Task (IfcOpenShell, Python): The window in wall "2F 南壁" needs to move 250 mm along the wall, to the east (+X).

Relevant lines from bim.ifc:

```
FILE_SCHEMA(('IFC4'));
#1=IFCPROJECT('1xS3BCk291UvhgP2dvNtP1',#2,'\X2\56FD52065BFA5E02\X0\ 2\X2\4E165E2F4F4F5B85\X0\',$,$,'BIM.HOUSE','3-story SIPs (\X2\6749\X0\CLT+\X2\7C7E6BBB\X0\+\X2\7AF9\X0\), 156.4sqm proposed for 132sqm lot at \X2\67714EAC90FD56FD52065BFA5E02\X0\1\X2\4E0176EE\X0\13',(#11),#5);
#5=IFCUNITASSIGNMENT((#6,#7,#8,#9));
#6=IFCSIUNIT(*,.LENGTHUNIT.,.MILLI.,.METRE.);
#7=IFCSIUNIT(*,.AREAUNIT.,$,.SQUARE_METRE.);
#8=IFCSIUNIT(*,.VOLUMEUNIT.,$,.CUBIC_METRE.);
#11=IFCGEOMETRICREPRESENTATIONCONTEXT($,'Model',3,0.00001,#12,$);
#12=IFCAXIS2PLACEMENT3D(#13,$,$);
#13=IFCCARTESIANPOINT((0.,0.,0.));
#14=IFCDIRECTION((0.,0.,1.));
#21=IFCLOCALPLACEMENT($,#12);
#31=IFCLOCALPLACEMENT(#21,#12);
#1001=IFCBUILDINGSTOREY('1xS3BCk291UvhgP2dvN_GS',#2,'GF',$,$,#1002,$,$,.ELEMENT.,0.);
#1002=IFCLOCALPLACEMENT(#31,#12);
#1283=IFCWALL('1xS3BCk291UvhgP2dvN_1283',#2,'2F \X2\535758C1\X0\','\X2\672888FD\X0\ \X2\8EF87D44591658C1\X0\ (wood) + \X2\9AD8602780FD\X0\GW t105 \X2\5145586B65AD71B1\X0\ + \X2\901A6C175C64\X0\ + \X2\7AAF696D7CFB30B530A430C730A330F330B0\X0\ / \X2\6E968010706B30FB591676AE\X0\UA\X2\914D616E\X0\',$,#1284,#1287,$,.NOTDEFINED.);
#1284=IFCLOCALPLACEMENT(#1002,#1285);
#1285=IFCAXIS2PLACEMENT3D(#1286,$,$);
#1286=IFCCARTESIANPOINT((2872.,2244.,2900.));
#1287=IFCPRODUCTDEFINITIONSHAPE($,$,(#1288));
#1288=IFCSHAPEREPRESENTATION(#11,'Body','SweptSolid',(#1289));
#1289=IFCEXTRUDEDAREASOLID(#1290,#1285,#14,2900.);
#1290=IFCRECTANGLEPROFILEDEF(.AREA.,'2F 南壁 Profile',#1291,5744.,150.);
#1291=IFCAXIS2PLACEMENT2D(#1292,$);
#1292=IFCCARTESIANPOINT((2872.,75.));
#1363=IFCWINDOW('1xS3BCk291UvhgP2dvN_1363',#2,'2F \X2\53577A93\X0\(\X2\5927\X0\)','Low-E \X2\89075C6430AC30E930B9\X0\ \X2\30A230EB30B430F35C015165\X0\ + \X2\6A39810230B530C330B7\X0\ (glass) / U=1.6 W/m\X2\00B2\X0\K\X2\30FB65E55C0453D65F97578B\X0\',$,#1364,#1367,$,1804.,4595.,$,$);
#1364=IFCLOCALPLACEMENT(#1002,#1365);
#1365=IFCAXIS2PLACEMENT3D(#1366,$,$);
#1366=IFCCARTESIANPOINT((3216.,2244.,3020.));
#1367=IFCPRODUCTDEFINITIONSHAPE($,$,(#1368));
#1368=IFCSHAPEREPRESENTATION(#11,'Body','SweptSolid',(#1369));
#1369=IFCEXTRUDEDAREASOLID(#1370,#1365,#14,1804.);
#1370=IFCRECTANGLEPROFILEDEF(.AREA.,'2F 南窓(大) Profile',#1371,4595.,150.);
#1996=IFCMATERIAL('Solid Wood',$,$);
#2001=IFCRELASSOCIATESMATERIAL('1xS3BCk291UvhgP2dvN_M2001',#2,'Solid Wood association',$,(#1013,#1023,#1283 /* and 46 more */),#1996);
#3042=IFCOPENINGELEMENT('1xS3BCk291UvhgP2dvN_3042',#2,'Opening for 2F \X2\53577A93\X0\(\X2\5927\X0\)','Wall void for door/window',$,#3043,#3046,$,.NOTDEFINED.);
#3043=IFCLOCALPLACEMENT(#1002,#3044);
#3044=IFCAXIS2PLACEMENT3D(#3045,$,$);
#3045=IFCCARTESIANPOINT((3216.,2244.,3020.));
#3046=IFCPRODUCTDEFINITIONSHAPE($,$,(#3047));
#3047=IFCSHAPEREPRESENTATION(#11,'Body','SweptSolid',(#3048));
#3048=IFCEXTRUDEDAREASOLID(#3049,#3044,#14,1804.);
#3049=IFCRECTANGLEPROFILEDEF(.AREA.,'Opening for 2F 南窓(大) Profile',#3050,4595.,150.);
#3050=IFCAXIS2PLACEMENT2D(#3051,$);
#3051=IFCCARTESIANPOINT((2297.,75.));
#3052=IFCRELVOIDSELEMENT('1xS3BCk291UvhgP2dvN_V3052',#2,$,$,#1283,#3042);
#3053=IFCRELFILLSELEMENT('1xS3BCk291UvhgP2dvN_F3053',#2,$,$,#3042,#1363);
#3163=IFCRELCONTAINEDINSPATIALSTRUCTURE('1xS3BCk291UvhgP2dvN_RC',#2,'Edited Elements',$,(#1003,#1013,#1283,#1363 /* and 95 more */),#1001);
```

```python
import ifcopenshell
import ifcopenshell.api.geometry
import ifcopenshell.util.placement
import ifcopenshell.util.unit

model = ifcopenshell.open("bim.ifc")
unit_scale = ifcopenshell.util.unit.calculate_unit_scale(model)

window = model.by_guid("1xS3BCk291UvhgP2dvN_1363")
opening = window.FillsVoids[0].RelatingOpeningElement
wall = opening.VoidsElements[0].RelatingBuildingElement

wall_matrix = ifcopenshell.util.placement.get_local_placement(wall.ObjectPlacement)
shift = wall_matrix[:3, 0] * 0.25 / unit_scale
before = ifcopenshell.util.placement.get_local_placement(window.ObjectPlacement)[:3, 3].copy()

# The window is not placed relative to its opening, so move both.
for product in (opening, window):
    matrix = ifcopenshell.util.placement.get_local_placement(product.ObjectPlacement)
    matrix[:3, 3] += shift
    ifcopenshell.api.geometry.edit_object_placement(model, product=product, matrix=matrix, is_si=False)

after = ifcopenshell.util.placement.get_local_placement(window.ObjectPlacement)[:3, 3]
print("window moved by", (after - before).round(3) + 0.0)

model.write("bim_edited.ifc")
```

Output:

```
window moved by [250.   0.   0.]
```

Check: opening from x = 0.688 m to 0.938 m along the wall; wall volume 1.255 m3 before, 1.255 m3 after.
